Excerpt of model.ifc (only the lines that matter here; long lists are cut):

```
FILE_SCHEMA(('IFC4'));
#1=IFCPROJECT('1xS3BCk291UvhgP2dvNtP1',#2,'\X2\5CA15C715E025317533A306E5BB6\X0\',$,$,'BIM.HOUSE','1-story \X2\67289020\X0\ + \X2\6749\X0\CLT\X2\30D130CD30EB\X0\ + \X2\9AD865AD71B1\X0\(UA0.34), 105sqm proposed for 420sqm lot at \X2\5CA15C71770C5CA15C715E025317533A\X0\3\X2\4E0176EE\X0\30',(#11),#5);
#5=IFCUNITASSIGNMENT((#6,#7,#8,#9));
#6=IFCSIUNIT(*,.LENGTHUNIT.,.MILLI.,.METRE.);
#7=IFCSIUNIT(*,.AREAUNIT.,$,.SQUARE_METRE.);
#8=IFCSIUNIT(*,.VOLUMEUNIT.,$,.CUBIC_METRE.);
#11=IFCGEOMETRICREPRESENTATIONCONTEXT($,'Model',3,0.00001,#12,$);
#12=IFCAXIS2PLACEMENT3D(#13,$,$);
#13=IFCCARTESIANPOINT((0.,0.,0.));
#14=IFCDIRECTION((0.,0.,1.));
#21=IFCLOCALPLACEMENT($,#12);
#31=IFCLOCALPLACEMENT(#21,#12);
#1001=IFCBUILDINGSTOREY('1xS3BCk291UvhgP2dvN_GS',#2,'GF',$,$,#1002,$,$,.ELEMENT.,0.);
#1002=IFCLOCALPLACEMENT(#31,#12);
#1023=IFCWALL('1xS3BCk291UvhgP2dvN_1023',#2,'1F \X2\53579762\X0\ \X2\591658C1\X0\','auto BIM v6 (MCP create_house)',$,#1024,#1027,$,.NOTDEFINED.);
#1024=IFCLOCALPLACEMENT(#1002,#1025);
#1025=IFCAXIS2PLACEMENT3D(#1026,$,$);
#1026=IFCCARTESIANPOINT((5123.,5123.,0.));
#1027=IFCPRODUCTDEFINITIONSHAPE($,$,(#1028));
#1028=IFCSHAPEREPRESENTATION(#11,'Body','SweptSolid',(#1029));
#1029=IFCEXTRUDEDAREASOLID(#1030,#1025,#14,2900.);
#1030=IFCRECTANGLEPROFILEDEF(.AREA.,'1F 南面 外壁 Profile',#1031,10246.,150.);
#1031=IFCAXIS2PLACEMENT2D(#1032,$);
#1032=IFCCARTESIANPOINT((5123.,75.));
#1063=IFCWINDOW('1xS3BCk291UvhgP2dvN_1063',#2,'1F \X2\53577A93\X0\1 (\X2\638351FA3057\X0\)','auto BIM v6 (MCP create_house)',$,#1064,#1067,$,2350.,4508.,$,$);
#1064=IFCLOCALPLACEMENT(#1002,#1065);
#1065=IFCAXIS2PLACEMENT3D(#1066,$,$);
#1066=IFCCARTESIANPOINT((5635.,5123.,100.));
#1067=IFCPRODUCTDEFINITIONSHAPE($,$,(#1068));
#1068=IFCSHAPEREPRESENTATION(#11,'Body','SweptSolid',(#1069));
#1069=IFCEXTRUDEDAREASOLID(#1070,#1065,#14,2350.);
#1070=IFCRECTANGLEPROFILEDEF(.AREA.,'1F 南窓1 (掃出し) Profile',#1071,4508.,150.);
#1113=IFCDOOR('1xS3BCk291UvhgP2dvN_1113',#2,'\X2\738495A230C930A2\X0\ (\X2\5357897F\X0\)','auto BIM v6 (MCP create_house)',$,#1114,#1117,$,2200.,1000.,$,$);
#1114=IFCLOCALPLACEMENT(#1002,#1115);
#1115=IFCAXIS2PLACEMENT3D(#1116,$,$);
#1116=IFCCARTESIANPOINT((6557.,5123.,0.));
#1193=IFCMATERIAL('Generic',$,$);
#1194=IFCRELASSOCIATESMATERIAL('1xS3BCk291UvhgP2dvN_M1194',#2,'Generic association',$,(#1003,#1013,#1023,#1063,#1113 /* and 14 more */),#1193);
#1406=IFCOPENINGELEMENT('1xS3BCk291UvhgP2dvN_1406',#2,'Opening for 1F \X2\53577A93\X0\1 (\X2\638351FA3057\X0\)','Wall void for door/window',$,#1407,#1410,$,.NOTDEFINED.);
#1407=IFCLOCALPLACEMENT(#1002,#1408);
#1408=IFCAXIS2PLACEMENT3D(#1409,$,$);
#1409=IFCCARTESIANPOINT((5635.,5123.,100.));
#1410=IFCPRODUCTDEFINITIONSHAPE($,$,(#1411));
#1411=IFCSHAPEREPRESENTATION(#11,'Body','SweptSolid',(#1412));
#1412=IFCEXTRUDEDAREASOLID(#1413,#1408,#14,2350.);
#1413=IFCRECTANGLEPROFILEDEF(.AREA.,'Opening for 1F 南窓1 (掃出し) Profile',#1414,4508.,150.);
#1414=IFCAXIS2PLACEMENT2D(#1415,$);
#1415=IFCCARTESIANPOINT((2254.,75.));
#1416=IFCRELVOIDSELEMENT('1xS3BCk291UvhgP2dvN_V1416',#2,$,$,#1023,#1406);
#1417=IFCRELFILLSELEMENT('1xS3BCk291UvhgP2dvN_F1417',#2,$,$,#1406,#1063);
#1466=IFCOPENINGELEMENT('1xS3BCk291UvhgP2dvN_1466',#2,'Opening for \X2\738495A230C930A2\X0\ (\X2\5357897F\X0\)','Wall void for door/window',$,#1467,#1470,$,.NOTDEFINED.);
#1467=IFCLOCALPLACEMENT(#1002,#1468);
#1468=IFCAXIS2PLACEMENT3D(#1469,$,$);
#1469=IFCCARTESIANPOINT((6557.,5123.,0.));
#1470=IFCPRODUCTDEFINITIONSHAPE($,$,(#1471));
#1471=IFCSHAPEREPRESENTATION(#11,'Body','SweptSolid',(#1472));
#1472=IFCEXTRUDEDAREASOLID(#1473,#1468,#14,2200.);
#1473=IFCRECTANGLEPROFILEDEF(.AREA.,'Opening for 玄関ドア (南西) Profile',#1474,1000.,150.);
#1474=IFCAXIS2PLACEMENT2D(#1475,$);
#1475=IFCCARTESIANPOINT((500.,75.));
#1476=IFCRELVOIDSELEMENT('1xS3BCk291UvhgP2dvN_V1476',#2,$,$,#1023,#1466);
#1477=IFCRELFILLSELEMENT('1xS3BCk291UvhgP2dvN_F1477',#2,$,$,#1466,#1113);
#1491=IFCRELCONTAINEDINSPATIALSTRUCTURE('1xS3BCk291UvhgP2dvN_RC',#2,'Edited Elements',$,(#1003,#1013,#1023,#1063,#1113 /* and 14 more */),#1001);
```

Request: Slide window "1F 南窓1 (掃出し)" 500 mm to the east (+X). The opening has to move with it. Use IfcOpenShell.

```python
import ifcopenshell
import ifcopenshell.api.geometry
import ifcopenshell.util.placement

model = ifcopenshell.open("model.ifc")

window = model.by_guid("1xS3BCk291UvhgP2dvN_1063")
opening = window.FillsVoids[0].RelatingOpeningElement
wall = opening.VoidsElements[0].RelatingBuildingElement

wall_matrix = ifcopenshell.util.placement.get_local_placement(wall.ObjectPlacement)
shift = wall_matrix[:3, 0] * 500.0
before = ifcopenshell.util.placement.get_local_placement(window.ObjectPlacement)[:3, 3].copy()

# The window is not placed relative to its opening, so move both.
for product in (opening, window):
    matrix = ifcopenshell.util.placement.get_local_placement(product.ObjectPlacement)
    matrix[:3, 3] += shift
    ifcopenshell.api.geometry.edit_object_placement(model, product=product, matrix=matrix, is_si=False)

after = ifcopenshell.util.placement.get_local_placement(window.ObjectPlacement)[:3, 3]
print("window moved by", (after - before).round(3) + 0.0)

model.write("model_rev.ifc")
```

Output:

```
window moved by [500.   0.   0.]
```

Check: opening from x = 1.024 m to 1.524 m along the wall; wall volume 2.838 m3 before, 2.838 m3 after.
